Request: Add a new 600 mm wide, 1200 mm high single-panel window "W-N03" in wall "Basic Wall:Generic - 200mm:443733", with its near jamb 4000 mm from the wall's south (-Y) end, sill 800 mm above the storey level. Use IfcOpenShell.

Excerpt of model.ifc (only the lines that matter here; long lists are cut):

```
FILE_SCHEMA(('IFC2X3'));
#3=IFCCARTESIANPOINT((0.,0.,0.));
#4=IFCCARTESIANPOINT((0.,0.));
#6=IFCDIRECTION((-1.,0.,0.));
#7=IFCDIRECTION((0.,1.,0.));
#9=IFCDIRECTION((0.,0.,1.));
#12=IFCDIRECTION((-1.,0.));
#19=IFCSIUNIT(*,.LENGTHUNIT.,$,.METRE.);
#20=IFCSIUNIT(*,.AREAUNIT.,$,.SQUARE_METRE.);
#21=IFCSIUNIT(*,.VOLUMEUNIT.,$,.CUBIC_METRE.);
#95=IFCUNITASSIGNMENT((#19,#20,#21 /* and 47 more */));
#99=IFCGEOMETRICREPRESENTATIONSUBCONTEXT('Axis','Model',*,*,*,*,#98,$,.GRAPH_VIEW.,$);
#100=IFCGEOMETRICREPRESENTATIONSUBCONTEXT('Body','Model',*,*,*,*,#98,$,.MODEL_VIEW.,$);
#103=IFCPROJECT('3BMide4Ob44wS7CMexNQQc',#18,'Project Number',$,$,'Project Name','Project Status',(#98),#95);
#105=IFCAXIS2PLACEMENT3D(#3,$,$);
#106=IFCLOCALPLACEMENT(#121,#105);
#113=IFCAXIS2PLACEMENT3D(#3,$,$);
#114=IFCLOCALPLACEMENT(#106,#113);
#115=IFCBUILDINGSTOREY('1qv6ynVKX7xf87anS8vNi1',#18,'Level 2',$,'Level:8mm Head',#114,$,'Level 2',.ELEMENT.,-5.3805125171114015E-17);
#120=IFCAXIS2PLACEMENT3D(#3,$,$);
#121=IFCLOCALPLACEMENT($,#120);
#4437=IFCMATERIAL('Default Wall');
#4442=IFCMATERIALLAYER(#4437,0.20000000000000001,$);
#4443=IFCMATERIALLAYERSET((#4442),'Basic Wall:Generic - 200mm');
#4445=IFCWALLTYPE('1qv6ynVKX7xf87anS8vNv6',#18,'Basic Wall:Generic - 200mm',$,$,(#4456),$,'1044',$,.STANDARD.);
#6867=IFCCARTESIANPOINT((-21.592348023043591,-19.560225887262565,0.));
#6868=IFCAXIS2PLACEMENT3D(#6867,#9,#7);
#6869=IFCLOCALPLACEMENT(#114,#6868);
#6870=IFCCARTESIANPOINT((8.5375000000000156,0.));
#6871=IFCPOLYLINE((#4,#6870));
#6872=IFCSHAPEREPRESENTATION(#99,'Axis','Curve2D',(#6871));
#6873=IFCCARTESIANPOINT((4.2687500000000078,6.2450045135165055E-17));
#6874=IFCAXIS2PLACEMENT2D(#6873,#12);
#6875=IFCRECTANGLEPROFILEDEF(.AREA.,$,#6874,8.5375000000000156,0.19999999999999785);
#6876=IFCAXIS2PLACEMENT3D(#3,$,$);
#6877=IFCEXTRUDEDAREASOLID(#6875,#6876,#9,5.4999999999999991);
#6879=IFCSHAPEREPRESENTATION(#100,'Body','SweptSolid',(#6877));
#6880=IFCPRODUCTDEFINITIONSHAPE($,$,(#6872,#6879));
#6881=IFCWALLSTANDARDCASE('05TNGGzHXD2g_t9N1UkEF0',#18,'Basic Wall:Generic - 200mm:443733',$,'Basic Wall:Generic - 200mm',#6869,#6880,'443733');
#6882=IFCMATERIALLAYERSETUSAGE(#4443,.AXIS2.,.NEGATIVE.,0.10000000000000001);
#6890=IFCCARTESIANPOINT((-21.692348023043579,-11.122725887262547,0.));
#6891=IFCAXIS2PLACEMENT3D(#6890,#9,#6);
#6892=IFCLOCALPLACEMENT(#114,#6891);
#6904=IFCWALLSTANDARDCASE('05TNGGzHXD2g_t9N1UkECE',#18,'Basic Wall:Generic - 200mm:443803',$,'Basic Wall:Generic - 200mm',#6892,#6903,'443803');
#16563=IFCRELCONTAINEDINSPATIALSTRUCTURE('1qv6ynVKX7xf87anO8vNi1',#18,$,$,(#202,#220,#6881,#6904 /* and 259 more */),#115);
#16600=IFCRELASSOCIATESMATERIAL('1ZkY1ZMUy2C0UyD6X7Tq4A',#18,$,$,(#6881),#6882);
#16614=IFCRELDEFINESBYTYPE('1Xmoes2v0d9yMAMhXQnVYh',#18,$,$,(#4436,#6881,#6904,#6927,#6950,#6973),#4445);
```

```python
import numpy as np
import ifcopenshell
import ifcopenshell.api.feature
import ifcopenshell.api.geometry
import ifcopenshell.api.root
import ifcopenshell.api.spatial
import ifcopenshell.api.type
import ifcopenshell.geom
import ifcopenshell.util.element
import ifcopenshell.util.placement
import ifcopenshell.util.representation
import ifcopenshell.util.shape
import ifcopenshell.util.unit

model = ifcopenshell.open("model.ifc")
unit_scale = ifcopenshell.util.unit.calculate_unit_scale(model)
settings = ifcopenshell.geom.settings()


def volume(element):
    """Net volume in cubic metres, openings subtracted."""
    shape = ifcopenshell.geom.create_shape(settings, element)
    return ifcopenshell.util.shape.get_volume(shape.geometry)


wall = model.by_guid("05TNGGzHXD2g_t9N1UkEF0")
storey = ifcopenshell.util.element.get_container(wall, ifc_class="IfcBuildingStorey")
context = ifcopenshell.util.representation.get_context(model, "Model", "Body", "MODEL_VIEW")
before = volume(wall)

width, height, from_end, sill = 0.6, 1.2, 4, 0.8  # metres

# The wall runs along its own X axis, and the end named is its -X end.
wall_shape = ifcopenshell.geom.create_shape(settings, wall)
x, y, z = ifcopenshell.util.shape.get_vertices(wall_shape.geometry).T
start = x.min() + from_end
face, thickness = float(y.min()), float(y.max() - y.min())
wall_matrix = ifcopenshell.util.placement.get_local_placement(wall.ObjectPlacement)
level = ifcopenshell.util.placement.get_local_placement(storey.ObjectPlacement)[2, 3]


def in_wall(x, y):
    """Placement at x, y metres in the wall's axes, at sill height."""
    matrix = wall_matrix.copy()
    matrix[:, 3] = wall_matrix @ np.array([x / unit_scale, y / unit_scale, 0.0, 1.0])
    matrix[2, 3] = level + sill / unit_scale
    return matrix


# Opening: a box that overshoots both wall faces by 50 mm.
opening = ifcopenshell.api.root.create_entity(model, ifc_class="IfcOpeningElement")
box = ifcopenshell.api.geometry.add_wall_representation(
    model, context=context, length=width, height=height, thickness=thickness + 0.1
)
ifcopenshell.api.geometry.assign_representation(model, product=opening, representation=box)
ifcopenshell.api.geometry.edit_object_placement(model, product=opening, matrix=in_wall(start, face - 0.05), is_si=False)
ifcopenshell.api.feature.add_feature(model, feature=opening, element=wall)

window = ifcopenshell.api.root.create_entity(model, ifc_class="IfcWindow", name="W-N03")
window.OverallWidth, window.OverallHeight = width / unit_scale, height / unit_scale
body = ifcopenshell.api.geometry.add_window_representation(
    model,
    context=context,
    overall_width=window.OverallWidth,
    overall_height=window.OverallHeight,
    partition_type="SINGLE_PANEL",
)
ifcopenshell.api.geometry.assign_representation(model, product=window, representation=body)
ifcopenshell.api.spatial.assign_container(model, products=[window], relating_structure=storey)
fills = ifcopenshell.api.feature.add_filling(model, opening=opening, element=window)
fills.OwnerHistory = window.OwnerHistory  # required in IFC2X3

# IFC2X3 keeps the operation on the window style.
style = ifcopenshell.api.root.create_entity(model, ifc_class="IfcWindowStyle", name="W-N03")
style.OperationType, style.ConstructionType = "SINGLE_PANEL", "NOTDEFINED"
style.ParameterTakesPrecedence = style.Sizeable = False
ifcopenshell.api.type.assign_type(model, related_objects=[window], relating_type=style)

# Centre the window in the wall's thickness.
ifcopenshell.api.geometry.edit_object_placement(model, product=window, matrix=in_wall(start, face), is_si=False)
window_shape = ifcopenshell.geom.create_shape(settings, window)
depth = ifcopenshell.util.shape.get_vertices(window_shape.geometry)[:, 1]
offset = face + thickness / 2 - (depth.min() + depth.max()) / 2
ifcopenshell.api.geometry.edit_object_placement(model, product=window, matrix=in_wall(start, offset), is_si=False)

after = volume(wall)

print(f"wall volume {before:.3f} -> {after:.3f} m3")

model.write("model_v2.ifc")
```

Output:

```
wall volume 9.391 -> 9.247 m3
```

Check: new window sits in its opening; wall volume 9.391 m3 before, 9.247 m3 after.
